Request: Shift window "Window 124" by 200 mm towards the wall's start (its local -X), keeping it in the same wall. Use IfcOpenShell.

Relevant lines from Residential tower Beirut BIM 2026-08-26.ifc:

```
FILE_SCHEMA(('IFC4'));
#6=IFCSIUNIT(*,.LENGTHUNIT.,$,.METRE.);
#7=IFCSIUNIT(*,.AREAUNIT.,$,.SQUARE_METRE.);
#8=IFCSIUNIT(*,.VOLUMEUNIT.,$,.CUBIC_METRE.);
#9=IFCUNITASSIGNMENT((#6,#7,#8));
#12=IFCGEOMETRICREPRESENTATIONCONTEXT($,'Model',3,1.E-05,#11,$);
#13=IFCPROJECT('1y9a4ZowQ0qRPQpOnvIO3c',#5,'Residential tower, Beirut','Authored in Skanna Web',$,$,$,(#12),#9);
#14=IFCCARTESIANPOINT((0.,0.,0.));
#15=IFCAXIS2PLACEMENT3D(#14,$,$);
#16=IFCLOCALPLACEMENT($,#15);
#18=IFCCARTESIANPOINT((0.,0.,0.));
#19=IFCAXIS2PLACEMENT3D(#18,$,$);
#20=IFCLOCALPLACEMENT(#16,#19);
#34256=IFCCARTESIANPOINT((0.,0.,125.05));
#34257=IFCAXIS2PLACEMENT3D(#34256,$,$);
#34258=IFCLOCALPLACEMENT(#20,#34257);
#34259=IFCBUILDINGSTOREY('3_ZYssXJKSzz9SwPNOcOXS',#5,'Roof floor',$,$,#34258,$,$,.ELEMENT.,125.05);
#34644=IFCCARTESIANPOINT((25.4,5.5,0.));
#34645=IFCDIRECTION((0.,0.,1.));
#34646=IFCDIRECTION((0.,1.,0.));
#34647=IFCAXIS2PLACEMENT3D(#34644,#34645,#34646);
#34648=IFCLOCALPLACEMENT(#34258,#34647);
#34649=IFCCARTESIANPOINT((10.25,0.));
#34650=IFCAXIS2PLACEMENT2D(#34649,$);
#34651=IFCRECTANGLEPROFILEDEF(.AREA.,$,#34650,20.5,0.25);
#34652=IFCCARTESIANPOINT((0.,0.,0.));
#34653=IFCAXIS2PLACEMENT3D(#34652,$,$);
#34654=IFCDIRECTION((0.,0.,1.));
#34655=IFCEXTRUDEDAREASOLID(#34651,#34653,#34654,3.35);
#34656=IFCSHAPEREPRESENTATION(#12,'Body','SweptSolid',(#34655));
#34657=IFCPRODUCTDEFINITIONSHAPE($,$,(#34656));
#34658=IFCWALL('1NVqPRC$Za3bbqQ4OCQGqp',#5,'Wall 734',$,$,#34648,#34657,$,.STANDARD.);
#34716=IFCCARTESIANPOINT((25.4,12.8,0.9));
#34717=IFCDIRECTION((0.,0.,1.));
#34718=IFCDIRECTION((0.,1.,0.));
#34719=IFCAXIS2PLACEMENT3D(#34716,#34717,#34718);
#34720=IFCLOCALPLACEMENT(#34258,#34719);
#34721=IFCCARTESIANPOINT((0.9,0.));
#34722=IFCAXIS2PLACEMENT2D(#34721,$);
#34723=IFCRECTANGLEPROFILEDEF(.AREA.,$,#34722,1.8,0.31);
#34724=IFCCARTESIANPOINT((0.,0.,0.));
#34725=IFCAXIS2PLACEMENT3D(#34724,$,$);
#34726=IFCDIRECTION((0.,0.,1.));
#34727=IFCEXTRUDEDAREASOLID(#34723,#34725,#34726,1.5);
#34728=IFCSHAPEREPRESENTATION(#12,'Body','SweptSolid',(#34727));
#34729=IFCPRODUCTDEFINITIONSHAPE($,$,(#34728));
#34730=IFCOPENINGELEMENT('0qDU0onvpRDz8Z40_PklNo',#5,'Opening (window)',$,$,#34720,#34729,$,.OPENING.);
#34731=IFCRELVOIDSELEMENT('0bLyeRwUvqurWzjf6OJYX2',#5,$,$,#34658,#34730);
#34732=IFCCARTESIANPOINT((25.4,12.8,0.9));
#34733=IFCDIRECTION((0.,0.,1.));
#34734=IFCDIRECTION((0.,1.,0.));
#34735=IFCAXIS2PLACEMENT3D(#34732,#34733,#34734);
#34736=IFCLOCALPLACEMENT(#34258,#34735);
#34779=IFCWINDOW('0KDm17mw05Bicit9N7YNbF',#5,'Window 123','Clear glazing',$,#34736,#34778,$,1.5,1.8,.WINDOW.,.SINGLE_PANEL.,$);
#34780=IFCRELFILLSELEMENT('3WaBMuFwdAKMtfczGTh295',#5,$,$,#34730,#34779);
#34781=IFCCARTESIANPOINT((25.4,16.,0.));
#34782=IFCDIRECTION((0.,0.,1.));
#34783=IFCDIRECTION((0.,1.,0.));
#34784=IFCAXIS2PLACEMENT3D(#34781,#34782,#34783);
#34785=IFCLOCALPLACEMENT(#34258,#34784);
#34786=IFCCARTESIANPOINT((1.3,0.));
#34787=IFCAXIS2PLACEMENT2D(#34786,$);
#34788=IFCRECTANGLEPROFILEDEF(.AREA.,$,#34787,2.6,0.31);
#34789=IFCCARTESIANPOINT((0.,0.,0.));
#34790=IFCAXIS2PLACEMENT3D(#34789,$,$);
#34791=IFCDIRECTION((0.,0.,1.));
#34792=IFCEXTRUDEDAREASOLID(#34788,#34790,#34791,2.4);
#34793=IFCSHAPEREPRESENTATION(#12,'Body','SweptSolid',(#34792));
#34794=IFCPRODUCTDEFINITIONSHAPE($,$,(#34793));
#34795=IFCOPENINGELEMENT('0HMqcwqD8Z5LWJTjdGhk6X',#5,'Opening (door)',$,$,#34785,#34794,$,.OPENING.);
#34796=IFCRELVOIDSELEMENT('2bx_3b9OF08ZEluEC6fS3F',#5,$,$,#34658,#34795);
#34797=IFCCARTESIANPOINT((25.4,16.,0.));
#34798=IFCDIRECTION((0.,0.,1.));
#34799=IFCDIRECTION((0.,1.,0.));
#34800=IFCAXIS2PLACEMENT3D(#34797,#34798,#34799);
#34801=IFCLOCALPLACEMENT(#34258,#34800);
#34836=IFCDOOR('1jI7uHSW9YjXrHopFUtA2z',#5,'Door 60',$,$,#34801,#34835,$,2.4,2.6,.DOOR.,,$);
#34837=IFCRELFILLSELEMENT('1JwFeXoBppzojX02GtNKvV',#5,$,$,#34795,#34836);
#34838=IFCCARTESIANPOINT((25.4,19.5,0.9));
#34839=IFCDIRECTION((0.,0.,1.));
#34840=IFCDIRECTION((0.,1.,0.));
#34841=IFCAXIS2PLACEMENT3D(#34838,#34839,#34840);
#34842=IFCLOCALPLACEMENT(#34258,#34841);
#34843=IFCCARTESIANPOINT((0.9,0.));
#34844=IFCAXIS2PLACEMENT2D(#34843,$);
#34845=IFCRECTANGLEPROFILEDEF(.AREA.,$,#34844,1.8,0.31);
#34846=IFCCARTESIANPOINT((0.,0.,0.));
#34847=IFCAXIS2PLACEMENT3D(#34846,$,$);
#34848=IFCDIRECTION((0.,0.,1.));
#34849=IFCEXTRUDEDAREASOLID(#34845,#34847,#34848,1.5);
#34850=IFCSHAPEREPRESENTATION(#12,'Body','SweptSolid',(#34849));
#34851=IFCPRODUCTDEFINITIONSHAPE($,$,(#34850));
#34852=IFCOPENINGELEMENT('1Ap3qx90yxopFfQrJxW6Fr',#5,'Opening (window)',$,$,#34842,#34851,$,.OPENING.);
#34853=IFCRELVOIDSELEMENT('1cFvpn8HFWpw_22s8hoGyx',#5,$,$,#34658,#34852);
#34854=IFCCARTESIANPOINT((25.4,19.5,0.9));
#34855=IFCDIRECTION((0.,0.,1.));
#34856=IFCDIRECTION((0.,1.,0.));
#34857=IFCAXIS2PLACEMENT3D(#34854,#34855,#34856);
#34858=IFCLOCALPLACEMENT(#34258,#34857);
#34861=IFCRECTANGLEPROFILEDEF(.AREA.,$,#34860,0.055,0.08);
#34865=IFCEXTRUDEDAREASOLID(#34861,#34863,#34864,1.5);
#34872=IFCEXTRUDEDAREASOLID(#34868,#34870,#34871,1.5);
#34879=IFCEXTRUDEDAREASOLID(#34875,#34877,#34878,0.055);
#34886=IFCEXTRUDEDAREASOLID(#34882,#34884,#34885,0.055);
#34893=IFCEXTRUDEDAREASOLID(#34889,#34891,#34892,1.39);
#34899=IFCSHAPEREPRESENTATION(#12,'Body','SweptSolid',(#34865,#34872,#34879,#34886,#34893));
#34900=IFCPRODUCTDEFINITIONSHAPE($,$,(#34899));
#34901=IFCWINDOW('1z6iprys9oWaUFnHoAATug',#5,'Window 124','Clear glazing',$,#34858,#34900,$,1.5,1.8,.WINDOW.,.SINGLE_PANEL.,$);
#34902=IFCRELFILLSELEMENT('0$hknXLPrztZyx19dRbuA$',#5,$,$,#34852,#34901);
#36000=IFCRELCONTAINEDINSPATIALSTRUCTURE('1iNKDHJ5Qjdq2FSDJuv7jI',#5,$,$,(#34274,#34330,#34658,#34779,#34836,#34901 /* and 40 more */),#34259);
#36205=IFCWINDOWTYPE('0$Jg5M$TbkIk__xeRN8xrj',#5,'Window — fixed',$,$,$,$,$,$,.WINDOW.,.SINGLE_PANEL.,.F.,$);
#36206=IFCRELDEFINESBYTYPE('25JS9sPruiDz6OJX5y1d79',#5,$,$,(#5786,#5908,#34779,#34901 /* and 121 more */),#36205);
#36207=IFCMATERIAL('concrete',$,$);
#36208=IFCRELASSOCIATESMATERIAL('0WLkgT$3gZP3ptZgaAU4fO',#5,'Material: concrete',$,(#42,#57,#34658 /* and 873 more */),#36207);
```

```python
import ifcopenshell
import ifcopenshell.api.geometry
import ifcopenshell.util.placement
import ifcopenshell.util.unit

model = ifcopenshell.open("Residential tower Beirut BIM 2026-08-26.ifc")
unit_scale = ifcopenshell.util.unit.calculate_unit_scale(model)

window = model.by_guid("1z6iprys9oWaUFnHoAATug")
opening = window.FillsVoids[0].RelatingOpeningElement
wall = opening.VoidsElements[0].RelatingBuildingElement

wall_matrix = ifcopenshell.util.placement.get_local_placement(wall.ObjectPlacement)
shift = wall_matrix[:3, 0] * -0.2 / unit_scale
before = ifcopenshell.util.placement.get_local_placement(window.ObjectPlacement)[:3, 3].copy()

# The window is not placed relative to its opening, so move both.
for product in (opening, window):
    matrix = ifcopenshell.util.placement.get_local_placement(product.ObjectPlacement)
    matrix[:3, 3] += shift
    ifcopenshell.api.geometry.edit_object_placement(model, product=product, matrix=matrix, is_si=False)

after = ifcopenshell.util.placement.get_local_placement(window.ObjectPlacement)[:3, 3]
print("window moved by", (after - before).round(3) + 0.0)

model.write("Residential tower Beirut BIM 2026-08-26_edited.ifc")
```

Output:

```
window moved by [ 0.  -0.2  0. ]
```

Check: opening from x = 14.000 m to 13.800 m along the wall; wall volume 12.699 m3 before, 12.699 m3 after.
